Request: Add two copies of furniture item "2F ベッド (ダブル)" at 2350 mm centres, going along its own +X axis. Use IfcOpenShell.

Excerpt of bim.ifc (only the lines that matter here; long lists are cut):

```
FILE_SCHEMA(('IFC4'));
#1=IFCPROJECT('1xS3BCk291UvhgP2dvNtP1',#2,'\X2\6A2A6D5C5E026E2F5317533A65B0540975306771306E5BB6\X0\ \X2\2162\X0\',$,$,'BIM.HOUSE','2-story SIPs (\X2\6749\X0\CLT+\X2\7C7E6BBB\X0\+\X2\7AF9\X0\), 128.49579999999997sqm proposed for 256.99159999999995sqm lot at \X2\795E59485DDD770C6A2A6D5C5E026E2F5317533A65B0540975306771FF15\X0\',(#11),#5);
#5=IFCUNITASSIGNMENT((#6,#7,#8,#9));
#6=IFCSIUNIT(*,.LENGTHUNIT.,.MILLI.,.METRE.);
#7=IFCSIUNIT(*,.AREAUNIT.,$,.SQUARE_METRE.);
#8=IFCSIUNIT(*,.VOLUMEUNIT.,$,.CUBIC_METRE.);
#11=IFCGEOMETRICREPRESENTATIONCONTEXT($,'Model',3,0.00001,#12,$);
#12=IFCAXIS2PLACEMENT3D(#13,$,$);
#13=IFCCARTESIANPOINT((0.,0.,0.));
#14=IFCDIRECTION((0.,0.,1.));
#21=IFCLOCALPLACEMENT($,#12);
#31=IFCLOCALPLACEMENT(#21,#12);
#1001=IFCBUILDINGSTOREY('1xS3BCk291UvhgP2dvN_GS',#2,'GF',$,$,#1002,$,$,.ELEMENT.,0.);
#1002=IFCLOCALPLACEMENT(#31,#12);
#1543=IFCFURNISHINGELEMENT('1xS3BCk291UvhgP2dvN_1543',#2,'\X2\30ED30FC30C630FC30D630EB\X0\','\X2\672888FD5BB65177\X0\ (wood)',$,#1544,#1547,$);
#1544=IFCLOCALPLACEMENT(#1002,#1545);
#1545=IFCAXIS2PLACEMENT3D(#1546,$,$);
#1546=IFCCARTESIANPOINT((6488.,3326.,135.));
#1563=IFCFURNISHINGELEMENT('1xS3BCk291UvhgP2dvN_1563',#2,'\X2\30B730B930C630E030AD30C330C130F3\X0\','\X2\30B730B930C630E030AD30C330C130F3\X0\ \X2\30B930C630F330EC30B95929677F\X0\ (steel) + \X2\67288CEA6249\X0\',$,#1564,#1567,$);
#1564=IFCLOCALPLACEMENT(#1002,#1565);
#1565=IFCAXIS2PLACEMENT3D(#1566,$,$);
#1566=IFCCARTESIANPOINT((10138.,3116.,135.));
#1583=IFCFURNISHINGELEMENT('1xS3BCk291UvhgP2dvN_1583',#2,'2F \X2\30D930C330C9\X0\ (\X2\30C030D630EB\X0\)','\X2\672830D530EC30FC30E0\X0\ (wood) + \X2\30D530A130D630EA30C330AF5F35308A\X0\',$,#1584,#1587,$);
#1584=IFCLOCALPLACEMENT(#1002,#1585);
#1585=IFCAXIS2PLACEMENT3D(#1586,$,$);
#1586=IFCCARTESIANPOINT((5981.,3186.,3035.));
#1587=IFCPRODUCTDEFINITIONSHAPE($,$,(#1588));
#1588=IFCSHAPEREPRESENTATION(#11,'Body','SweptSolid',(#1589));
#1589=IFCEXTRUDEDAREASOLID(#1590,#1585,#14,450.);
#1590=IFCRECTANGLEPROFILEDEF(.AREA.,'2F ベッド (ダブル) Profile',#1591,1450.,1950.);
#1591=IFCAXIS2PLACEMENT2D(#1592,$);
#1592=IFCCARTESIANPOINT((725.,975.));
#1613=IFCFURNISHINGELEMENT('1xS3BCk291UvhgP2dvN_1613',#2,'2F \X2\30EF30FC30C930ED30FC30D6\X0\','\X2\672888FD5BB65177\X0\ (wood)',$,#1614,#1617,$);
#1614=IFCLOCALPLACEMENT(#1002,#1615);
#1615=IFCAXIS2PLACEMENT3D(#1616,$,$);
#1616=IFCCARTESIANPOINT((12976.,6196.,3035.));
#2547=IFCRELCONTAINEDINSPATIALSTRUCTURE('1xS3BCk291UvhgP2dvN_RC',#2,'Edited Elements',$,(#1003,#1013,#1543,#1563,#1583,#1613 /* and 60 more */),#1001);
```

```python
import ifcopenshell
import ifcopenshell.api.geometry
import ifcopenshell.api.root
import ifcopenshell.util.element
import ifcopenshell.util.placement
import ifcopenshell.util.unit

model = ifcopenshell.open("bim.ifc")
unit_scale = ifcopenshell.util.unit.calculate_unit_scale(model)


def reuse_history(source, copy):
    """copy_class also copies each property set's owner history, people and application; keep the originals."""
    for rel in copy.IsDefinedBy:
        if rel.is_a("IfcRelDefinesByProperties") and (history := rel.RelatingPropertyDefinition.OwnerHistory):
            rel.RelatingPropertyDefinition.OwnerHistory = source.OwnerHistory
            ifcopenshell.util.element.remove_deep2(model, history)


source = model.by_guid("1xS3BCk291UvhgP2dvN_1583")
base = ifcopenshell.util.placement.get_local_placement(source.ObjectPlacement)
step = base[:3, 0] * 2.35 / unit_scale

for i in range(1, 3):
    copy = ifcopenshell.api.root.copy_class(model, product=source)
    copy.Representation = ifcopenshell.util.element.copy_deep(
        model, source.Representation, exclude=["IfcGeometricRepresentationContext", "IfcRepresentationMap"]
    )
    reuse_history(source, copy)
    matrix = base.copy()
    matrix[:3, 3] += i * step
    print("added at", matrix[:3, 3].round(3) + 0.0)
    ifcopenshell.api.geometry.edit_object_placement(model, product=copy, matrix=matrix, is_si=False)

model.write("bim_v2.ifc")
```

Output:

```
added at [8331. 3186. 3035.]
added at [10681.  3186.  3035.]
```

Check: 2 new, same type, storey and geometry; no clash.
